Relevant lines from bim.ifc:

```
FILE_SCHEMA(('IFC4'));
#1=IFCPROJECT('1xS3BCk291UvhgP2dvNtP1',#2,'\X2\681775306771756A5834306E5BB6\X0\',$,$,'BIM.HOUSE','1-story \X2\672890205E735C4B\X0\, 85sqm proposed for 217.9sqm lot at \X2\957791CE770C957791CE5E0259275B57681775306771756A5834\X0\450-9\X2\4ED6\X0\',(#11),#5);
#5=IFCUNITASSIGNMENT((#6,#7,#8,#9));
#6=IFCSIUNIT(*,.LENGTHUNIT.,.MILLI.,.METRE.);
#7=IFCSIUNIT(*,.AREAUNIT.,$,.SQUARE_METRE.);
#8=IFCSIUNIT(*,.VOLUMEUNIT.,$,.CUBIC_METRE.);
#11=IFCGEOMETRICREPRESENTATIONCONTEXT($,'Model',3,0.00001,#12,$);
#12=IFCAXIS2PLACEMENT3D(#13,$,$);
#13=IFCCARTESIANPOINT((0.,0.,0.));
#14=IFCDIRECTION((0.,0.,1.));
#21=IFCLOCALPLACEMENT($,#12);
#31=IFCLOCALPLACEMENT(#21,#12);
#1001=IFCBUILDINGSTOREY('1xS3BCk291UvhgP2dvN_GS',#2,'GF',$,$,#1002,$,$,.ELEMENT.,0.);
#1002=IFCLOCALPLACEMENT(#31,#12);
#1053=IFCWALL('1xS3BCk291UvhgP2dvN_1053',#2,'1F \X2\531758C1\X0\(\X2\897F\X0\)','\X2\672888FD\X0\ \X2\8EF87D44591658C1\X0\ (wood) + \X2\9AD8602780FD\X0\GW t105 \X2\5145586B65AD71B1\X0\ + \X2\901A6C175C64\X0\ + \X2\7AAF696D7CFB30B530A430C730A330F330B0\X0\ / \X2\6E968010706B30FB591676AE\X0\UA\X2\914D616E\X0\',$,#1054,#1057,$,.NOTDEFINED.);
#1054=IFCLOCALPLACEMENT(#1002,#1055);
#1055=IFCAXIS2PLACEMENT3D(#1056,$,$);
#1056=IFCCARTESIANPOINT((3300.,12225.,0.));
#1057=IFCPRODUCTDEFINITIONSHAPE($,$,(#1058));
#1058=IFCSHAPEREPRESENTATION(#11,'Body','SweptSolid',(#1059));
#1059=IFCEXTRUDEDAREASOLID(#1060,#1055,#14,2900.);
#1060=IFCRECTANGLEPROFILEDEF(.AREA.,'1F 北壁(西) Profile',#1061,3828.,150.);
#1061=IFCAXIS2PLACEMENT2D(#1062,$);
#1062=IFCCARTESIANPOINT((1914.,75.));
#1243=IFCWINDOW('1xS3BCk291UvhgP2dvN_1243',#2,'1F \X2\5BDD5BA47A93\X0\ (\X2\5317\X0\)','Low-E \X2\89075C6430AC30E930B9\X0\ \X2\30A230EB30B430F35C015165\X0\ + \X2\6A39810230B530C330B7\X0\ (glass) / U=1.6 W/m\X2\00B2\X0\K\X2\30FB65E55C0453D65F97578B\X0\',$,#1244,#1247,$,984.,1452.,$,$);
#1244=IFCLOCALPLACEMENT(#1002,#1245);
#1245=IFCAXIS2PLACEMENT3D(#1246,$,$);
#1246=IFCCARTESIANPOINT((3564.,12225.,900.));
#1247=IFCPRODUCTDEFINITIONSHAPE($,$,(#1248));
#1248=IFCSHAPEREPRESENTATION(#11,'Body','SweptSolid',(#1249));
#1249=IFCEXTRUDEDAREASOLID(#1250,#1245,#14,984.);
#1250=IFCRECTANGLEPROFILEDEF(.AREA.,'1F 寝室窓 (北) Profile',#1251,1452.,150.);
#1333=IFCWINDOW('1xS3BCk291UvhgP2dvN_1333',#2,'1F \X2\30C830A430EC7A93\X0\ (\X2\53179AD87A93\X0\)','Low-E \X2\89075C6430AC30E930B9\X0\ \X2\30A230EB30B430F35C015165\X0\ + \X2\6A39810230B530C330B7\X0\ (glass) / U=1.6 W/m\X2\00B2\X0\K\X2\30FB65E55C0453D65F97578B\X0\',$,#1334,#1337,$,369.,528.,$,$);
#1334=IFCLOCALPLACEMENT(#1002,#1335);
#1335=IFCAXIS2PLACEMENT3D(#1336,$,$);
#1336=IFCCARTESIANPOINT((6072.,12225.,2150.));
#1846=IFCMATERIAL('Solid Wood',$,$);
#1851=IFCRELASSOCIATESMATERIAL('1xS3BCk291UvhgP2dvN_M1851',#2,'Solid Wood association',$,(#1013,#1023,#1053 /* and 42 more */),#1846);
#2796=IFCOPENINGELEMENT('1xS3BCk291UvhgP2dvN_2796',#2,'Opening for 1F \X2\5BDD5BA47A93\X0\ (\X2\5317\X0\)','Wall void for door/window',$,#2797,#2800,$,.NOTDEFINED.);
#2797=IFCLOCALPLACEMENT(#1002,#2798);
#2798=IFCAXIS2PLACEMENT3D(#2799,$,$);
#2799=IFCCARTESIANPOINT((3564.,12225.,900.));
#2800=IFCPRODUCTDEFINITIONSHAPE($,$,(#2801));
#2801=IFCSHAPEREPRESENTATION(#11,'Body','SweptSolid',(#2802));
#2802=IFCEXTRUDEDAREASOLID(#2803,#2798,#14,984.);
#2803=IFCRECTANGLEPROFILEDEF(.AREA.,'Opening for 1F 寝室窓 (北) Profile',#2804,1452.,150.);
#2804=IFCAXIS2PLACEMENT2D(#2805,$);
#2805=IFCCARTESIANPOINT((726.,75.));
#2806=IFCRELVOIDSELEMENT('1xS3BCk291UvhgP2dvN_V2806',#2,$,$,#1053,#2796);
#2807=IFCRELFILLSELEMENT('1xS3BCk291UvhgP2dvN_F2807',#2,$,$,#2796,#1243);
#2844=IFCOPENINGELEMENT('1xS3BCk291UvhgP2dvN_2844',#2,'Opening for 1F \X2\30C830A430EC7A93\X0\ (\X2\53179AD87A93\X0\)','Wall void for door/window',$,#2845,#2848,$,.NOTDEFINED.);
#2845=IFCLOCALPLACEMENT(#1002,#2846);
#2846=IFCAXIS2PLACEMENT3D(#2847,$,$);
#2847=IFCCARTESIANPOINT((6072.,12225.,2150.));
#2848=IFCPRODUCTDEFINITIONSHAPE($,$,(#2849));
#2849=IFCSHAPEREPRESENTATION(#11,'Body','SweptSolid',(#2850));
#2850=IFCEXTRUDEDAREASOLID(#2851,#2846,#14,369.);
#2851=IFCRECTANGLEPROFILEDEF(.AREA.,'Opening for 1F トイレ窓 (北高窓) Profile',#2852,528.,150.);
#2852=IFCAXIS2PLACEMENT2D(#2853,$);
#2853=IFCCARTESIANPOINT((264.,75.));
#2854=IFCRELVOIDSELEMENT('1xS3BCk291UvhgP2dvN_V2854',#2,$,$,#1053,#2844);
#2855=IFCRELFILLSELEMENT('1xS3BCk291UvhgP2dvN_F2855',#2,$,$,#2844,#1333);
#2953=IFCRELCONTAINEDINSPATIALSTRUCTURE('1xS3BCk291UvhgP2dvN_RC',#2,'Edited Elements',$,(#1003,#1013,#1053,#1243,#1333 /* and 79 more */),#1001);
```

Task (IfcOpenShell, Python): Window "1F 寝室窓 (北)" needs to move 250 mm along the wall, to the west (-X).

```python
import ifcopenshell
import ifcopenshell.api.geometry
import ifcopenshell.util.placement

model = ifcopenshell.open("bim.ifc")

window = model.by_id(1243)
opening = window.FillsVoids[0].RelatingOpeningElement
wall = opening.VoidsElements[0].RelatingBuildingElement

wall_matrix = ifcopenshell.util.placement.get_local_placement(wall.ObjectPlacement)
shift = wall_matrix[:3, 0] * -250.0
before = ifcopenshell.util.placement.get_local_placement(window.ObjectPlacement)[:3, 3].copy()

# The window is not placed relative to its opening, so move both.
for product in (opening, window):
    matrix = ifcopenshell.util.placement.get_local_placement(product.ObjectPlacement)
    matrix[:3, 3] += shift
    ifcopenshell.api.geometry.edit_object_placement(model, product=product, matrix=matrix, is_si=False)

after = ifcopenshell.util.placement.get_local_placement(window.ObjectPlacement)[:3, 3]
print("window moved by", (after - before).round(3) + 0.0)

model.write("bim-out.ifc")
```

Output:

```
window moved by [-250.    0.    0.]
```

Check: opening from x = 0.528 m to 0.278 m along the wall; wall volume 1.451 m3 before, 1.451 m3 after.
